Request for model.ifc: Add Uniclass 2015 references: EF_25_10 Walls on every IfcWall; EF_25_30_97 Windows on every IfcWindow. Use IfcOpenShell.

First a look at what the model holds.

```python
import ifcopenshell

model = ifcopenshell.open("model.ifc")
print(model.schema)
print("classifications:", [c.Name for c in model.by_type("IfcClassification")])
for ifc_class in ("IfcDoor", "IfcRoof", "IfcStair", "IfcWall", "IfcWindow"):
    print(ifc_class, len(model.by_type(ifc_class)))
```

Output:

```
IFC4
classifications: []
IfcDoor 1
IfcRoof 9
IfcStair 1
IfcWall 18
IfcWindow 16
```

```python
import ifcopenshell
import ifcopenshell.api.classification

model = ifcopenshell.open("model.ifc")

system = ifcopenshell.api.classification.add_classification(model, classification="Uniclass 2015")

codes = {
    "IfcWall": ("EF_25_10", "Walls"),
    "IfcWindow": ("EF_25_30_97", "Windows"),
}
for ifc_class, (code, name) in codes.items():
    products = model.by_type(ifc_class)
    ifcopenshell.api.classification.add_reference(
        model, products=products, classification=system, identification=code, name=name
    )
    print(code, len(products))

model.write("model-out.ifc")
```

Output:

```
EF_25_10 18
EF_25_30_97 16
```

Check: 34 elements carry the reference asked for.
